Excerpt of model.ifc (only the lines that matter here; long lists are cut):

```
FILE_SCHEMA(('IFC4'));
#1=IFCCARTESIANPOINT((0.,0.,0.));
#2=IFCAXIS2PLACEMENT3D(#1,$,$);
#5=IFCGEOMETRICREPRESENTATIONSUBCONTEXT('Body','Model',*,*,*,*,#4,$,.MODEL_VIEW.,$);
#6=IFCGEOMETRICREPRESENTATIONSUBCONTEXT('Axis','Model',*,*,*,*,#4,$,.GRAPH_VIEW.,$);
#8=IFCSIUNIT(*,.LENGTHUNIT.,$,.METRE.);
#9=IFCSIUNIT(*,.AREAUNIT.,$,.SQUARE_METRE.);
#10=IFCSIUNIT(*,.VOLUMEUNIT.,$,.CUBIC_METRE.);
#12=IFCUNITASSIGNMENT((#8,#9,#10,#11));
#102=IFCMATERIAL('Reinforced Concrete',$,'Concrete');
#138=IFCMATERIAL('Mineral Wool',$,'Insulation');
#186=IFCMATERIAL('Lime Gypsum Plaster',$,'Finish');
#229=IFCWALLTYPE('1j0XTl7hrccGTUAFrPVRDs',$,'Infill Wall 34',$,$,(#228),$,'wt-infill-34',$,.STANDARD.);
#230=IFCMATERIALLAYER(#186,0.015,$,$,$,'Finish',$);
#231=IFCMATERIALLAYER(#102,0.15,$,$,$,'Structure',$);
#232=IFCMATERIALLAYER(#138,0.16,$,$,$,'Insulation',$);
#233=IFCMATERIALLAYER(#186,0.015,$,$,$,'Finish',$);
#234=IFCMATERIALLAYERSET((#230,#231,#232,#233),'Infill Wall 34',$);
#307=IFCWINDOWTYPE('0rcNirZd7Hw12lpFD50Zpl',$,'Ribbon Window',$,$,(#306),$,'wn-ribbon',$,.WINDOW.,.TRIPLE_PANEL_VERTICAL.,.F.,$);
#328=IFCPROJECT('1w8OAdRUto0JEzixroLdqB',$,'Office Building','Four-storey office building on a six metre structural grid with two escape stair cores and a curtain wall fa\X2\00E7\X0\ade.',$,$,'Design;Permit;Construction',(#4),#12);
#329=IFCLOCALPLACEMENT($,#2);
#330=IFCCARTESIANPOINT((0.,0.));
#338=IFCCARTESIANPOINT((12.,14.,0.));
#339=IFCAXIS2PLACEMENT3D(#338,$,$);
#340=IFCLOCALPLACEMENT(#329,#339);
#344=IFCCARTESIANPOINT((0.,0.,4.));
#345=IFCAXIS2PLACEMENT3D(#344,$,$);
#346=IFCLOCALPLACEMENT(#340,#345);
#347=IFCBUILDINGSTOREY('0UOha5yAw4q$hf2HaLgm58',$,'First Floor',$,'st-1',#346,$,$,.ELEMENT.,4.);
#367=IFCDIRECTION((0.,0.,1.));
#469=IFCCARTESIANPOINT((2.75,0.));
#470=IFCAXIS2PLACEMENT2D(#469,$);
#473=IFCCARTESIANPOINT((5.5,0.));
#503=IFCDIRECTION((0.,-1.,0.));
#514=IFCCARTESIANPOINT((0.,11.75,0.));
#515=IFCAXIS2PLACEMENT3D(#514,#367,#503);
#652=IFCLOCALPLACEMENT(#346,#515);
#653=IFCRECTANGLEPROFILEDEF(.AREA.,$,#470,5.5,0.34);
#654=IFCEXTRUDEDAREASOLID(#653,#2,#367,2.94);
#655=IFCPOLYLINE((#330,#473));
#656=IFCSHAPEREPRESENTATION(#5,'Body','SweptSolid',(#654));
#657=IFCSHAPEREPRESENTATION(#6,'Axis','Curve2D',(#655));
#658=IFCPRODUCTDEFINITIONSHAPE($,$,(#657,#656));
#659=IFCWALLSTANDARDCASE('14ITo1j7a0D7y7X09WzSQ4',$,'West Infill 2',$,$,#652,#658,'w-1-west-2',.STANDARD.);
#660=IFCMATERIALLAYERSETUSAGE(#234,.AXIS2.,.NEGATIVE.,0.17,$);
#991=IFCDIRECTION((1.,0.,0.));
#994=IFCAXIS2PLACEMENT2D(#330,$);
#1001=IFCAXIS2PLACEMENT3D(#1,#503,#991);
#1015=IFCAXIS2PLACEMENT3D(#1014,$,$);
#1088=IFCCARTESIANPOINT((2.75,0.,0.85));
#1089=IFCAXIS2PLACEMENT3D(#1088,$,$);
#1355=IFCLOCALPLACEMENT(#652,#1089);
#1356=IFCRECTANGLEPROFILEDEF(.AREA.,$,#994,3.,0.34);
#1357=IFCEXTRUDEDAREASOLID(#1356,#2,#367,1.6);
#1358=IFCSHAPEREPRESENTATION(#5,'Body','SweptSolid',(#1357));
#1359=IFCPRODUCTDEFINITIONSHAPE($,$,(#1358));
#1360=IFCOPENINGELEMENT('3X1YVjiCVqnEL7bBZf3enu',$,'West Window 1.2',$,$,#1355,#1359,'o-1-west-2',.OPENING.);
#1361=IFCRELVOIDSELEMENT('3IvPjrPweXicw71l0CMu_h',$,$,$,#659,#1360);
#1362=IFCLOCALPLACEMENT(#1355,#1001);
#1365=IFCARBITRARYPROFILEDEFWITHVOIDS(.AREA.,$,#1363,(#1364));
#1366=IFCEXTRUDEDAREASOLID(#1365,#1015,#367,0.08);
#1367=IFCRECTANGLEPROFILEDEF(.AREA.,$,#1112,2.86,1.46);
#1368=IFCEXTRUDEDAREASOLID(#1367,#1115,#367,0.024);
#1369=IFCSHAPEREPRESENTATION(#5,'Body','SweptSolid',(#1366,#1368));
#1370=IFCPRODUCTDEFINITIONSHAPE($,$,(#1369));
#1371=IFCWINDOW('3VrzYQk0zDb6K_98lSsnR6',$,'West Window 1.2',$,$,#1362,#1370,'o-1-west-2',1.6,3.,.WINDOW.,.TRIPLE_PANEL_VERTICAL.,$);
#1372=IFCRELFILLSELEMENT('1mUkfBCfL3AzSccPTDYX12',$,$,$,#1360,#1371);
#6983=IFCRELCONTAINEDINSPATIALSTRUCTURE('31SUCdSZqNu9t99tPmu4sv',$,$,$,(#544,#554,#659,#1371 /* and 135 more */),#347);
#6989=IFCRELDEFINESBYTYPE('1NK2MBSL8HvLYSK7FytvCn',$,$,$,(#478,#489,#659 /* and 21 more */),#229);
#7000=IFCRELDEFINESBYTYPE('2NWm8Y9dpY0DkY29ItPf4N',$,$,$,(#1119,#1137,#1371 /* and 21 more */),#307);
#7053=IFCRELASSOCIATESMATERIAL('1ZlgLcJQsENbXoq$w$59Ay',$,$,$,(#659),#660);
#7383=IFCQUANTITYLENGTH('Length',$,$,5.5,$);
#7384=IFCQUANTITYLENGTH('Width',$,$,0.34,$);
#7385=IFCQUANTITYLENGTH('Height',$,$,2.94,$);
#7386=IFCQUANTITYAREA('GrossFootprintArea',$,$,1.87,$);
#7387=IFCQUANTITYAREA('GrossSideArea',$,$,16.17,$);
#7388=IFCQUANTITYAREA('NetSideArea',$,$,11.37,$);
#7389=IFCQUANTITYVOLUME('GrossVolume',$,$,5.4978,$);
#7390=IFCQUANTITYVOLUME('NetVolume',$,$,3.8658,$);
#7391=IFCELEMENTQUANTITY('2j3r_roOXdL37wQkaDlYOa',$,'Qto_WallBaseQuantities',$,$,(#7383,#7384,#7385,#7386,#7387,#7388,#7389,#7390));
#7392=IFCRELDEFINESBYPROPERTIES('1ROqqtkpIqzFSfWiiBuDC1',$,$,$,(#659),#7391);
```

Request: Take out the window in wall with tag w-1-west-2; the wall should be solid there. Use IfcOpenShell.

```python
import ifcopenshell
import ifcopenshell.api.feature
import ifcopenshell.api.pset
import ifcopenshell.api.root
import ifcopenshell.geom
import ifcopenshell.util.element
import ifcopenshell.util.shape
import ifcopenshell.util.unit

model = ifcopenshell.open("model.ifc")
area_scale = ifcopenshell.util.unit.calculate_unit_scale(model, "AREAUNIT")
volume_scale = ifcopenshell.util.unit.calculate_unit_scale(model, "VOLUMEUNIT")
settings = ifcopenshell.geom.settings()


def volume(element):
    """Net volume in cubic metres, openings subtracted."""
    shape = ifcopenshell.geom.create_shape(settings, element)
    return ifcopenshell.util.shape.get_volume(shape.geometry)


window = model.by_guid("3VrzYQk0zDb6K_98lSsnR6")
opening = window.FillsVoids[0].RelatingOpeningElement
wall = opening.VoidsElements[0].RelatingBuildingElement
before = volume(wall)

ifcopenshell.api.root.remove_product(model, product=window)
ifcopenshell.api.feature.remove_feature(model, feature=opening)

after = volume(wall)
thickness = 0.34  # wall thickness in metres

# Update the wall's stored quantities.
qto = model.by_id(ifcopenshell.util.element.get_pset(wall, "Qto_WallBaseQuantities", should_inherit=False)["id"])
ifcopenshell.api.pset.edit_qto(model, qto=qto, properties={
    "NetSideArea": after / thickness / area_scale,
    "NetVolume": after / volume_scale,
})

print(f"wall volume {before:.3f} -> {after:.3f} m3")

model.write("model_rev.ifc")
```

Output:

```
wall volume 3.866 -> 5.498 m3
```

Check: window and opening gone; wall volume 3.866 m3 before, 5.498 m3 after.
